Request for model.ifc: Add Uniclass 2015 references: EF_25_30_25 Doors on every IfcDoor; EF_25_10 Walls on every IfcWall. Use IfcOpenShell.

First a look at what the model holds.

```python
import ifcopenshell

model = ifcopenshell.open("model.ifc")
print(model.schema)
print("classifications:", [c.Name for c in model.by_type("IfcClassification")])
for ifc_class in ("IfcDoor", "IfcRoof", "IfcStair", "IfcWall", "IfcWindow"):
    print(ifc_class, len(model.by_type(ifc_class)))
```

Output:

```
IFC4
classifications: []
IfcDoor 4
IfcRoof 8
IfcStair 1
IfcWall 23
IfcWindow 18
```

```python
import ifcopenshell
import ifcopenshell.api.classification

model = ifcopenshell.open("model.ifc")

system = ifcopenshell.api.classification.add_classification(model, classification="Uniclass 2015")

codes = {
    "IfcDoor": ("EF_25_30_25", "Doors"),
    "IfcWall": ("EF_25_10", "Walls"),
}
for ifc_class, (code, name) in codes.items():
    products = model.by_type(ifc_class)
    ifcopenshell.api.classification.add_reference(
        model, products=products, classification=system, identification=code, name=name
    )
    print(code, len(products))

model.write("model_rev.ifc")
```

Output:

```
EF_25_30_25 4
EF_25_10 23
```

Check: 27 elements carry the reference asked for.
